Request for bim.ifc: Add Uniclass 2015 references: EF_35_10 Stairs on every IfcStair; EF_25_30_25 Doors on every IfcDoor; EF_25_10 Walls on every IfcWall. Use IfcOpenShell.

First a look at what the model holds.

```python
import ifcopenshell

model = ifcopenshell.open("bim.ifc")
print(model.schema)
print("classifications:", [c.Name for c in model.by_type("IfcClassification")])
for ifc_class in ("IfcDoor", "IfcRoof", "IfcStair", "IfcWall", "IfcWindow"):
    print(ifc_class, len(model.by_type(ifc_class)))
```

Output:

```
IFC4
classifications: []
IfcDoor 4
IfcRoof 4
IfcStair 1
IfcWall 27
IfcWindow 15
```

```python
import ifcopenshell
import ifcopenshell.api.classification

model = ifcopenshell.open("bim.ifc")

system = ifcopenshell.api.classification.add_classification(model, classification="Uniclass 2015")

codes = {
    "IfcStair": ("EF_35_10", "Stairs"),
    "IfcDoor": ("EF_25_30_25", "Doors"),
    "IfcWall": ("EF_25_10", "Walls"),
}
for ifc_class, (code, name) in codes.items():
    products = model.by_type(ifc_class)
    ifcopenshell.api.classification.add_reference(
        model, products=products, classification=system, identification=code, name=name
    )
    print(code, len(products))

model.write("bim-out.ifc")
```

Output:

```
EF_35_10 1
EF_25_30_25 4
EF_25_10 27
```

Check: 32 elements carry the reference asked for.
